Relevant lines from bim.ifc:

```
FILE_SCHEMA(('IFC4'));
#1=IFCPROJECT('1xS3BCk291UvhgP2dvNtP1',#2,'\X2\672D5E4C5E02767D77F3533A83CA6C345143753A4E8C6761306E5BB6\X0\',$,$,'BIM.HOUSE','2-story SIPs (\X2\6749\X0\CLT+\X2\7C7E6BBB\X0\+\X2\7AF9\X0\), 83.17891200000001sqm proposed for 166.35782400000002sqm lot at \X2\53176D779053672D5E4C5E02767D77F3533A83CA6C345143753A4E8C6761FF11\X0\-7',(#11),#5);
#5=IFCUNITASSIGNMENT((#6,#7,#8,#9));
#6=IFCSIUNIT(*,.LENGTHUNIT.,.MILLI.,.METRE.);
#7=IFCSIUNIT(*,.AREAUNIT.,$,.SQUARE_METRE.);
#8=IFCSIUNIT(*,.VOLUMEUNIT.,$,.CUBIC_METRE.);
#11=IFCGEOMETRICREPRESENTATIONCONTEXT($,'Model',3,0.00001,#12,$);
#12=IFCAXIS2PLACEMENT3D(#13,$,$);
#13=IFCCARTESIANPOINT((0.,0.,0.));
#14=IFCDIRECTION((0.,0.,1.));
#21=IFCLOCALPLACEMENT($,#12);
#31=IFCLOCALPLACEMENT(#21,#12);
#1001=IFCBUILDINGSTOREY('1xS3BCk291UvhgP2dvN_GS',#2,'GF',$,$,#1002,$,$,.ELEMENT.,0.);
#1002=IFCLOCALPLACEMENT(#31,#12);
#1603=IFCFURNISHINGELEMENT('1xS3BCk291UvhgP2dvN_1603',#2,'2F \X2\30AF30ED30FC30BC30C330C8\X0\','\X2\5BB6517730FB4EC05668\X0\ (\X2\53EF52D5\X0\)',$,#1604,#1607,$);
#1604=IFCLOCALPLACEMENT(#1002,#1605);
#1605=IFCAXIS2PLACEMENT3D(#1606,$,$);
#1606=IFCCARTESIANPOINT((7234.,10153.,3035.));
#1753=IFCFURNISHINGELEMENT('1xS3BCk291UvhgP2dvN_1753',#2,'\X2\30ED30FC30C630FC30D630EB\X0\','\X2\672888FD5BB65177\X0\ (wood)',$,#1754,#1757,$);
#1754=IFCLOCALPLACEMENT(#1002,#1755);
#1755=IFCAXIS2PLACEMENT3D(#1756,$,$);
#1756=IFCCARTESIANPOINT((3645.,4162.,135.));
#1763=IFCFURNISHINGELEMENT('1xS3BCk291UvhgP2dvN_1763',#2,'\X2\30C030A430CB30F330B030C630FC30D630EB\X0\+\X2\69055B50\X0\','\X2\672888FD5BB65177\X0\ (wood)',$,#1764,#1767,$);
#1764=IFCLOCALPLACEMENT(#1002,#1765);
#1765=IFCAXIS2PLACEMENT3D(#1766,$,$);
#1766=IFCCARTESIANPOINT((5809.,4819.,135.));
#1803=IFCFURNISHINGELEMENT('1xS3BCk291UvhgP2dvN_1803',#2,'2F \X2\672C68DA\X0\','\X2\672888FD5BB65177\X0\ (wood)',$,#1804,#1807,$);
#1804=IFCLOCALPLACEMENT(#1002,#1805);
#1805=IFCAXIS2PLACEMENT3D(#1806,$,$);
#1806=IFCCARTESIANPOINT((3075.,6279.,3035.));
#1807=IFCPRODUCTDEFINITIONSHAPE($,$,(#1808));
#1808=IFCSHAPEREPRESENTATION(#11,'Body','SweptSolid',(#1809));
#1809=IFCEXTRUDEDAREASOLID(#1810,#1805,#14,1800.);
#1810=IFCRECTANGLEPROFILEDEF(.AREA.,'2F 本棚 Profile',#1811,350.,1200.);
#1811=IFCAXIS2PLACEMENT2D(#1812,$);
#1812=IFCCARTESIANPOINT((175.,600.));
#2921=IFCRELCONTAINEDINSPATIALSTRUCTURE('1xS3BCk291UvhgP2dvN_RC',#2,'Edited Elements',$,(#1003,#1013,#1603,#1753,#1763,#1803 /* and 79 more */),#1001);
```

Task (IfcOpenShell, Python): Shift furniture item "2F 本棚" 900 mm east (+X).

```python
import ifcopenshell
import ifcopenshell.api.geometry
import ifcopenshell.util.placement
import ifcopenshell.util.unit

model = ifcopenshell.open("bim.ifc")
unit_scale = ifcopenshell.util.unit.calculate_unit_scale(model)

item = model.by_guid("1xS3BCk291UvhgP2dvN_1803")
matrix = ifcopenshell.util.placement.get_local_placement(item.ObjectPlacement)
matrix[0, 3] += 0.9 / unit_scale
ifcopenshell.api.geometry.edit_object_placement(model, product=item, matrix=matrix, is_si=False)

print(ifcopenshell.util.placement.get_local_placement(item.ObjectPlacement).round(3) + 0.0)

model.write("bim_updated.ifc")
```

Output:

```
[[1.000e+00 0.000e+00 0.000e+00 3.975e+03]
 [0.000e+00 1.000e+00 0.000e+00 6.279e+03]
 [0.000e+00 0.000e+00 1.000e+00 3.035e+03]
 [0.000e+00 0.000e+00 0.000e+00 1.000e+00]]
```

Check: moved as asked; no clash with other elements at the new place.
